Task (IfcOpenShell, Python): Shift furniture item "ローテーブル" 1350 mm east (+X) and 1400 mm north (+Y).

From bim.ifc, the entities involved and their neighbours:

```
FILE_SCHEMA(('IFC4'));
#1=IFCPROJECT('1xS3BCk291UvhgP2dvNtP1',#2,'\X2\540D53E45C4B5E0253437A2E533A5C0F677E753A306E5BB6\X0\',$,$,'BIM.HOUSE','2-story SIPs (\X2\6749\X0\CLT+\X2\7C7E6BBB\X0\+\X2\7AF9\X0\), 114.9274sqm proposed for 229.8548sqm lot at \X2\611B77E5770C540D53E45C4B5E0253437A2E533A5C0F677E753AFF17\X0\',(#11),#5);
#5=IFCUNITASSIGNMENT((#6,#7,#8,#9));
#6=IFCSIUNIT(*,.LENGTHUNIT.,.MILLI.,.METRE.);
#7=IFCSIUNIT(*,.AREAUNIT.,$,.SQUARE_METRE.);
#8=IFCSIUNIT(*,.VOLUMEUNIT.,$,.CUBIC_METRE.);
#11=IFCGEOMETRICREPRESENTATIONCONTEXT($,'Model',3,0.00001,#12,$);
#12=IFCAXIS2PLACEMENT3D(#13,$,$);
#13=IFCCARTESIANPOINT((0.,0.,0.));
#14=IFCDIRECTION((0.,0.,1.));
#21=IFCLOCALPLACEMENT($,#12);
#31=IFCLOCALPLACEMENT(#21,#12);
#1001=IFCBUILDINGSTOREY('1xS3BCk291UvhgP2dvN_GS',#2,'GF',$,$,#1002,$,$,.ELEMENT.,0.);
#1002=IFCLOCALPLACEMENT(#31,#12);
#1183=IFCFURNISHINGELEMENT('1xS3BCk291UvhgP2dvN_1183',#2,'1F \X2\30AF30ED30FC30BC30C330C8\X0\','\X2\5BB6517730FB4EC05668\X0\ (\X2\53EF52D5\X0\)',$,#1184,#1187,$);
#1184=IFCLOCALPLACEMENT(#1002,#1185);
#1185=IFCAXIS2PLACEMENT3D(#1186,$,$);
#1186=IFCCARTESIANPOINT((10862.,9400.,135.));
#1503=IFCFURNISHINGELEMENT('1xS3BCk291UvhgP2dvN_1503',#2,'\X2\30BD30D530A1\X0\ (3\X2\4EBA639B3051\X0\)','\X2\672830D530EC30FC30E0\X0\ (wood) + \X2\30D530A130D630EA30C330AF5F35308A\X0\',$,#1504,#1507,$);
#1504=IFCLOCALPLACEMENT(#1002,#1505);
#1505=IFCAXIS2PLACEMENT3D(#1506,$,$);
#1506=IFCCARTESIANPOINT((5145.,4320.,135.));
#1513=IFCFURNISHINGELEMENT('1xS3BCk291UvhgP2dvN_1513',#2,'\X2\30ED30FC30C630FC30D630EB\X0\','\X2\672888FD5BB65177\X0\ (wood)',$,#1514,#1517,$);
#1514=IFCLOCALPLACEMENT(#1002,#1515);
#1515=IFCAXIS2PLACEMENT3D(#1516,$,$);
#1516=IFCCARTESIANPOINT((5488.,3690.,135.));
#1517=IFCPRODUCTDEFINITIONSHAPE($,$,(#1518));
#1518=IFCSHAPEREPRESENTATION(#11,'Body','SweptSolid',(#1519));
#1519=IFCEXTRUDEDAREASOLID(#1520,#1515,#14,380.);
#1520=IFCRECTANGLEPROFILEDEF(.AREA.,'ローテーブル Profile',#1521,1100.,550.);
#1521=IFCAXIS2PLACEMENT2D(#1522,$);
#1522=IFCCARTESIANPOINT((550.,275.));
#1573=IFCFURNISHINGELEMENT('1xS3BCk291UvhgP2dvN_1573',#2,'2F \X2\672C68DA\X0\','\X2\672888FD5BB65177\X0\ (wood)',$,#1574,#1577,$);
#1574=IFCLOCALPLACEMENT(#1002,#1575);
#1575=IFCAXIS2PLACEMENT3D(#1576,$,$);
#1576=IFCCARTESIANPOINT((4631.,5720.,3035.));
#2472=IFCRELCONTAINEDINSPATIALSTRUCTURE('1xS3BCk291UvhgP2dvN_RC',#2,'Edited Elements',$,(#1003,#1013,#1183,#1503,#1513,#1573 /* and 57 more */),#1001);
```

```python
import ifcopenshell
import ifcopenshell.api.geometry
import ifcopenshell.util.placement
import ifcopenshell.util.unit

model = ifcopenshell.open("bim.ifc")
unit_scale = ifcopenshell.util.unit.calculate_unit_scale(model)

item = model.by_guid("1xS3BCk291UvhgP2dvN_1513")
matrix = ifcopenshell.util.placement.get_local_placement(item.ObjectPlacement)
matrix[0, 3] += 1.35 / unit_scale
matrix[1, 3] += 1.4 / unit_scale
ifcopenshell.api.geometry.edit_object_placement(model, product=item, matrix=matrix, is_si=False)

print(ifcopenshell.util.placement.get_local_placement(item.ObjectPlacement).round(3) + 0.0)

model.write("bim_updated.ifc")
```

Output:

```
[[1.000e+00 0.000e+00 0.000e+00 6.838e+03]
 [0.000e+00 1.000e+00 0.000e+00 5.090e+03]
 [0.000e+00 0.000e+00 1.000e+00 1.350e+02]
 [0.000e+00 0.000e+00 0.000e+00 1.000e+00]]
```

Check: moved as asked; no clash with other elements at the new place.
